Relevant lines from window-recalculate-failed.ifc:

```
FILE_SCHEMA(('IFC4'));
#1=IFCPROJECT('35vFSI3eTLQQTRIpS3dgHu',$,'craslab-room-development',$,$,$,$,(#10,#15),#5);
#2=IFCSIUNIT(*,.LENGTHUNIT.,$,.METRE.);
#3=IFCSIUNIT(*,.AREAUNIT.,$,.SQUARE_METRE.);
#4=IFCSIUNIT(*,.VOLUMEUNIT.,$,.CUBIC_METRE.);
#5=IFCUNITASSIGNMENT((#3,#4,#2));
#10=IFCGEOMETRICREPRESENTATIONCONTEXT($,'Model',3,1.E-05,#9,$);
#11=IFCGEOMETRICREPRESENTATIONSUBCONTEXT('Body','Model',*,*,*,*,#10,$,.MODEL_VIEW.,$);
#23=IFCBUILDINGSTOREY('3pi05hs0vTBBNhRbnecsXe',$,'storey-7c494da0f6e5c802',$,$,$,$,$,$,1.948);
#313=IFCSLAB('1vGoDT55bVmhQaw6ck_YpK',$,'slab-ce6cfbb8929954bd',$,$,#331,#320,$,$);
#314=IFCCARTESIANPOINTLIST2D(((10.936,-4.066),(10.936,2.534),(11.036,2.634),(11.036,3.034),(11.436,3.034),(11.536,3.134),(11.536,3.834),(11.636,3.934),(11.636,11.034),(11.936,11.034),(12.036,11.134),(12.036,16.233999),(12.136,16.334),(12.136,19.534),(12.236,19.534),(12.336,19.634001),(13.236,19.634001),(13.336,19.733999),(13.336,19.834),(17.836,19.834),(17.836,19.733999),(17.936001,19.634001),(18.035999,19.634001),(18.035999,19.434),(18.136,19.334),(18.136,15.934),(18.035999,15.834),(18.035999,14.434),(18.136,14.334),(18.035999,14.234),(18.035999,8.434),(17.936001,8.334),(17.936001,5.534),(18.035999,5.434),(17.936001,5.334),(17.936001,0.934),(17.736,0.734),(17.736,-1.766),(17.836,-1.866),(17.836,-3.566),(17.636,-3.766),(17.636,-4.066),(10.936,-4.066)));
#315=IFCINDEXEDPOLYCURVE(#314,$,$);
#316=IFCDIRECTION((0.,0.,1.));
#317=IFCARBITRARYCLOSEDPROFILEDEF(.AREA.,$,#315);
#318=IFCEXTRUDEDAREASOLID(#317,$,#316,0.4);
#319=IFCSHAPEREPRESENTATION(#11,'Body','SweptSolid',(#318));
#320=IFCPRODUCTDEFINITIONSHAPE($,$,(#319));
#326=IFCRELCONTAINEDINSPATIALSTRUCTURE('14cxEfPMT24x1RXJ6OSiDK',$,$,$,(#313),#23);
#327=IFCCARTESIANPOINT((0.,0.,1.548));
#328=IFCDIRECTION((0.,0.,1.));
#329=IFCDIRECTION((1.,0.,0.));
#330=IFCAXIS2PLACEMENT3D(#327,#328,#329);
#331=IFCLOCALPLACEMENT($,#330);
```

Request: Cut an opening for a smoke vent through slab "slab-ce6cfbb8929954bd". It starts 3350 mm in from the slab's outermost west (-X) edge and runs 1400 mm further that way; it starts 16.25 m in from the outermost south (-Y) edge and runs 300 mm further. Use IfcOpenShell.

```python
import numpy as np
import ifcopenshell
import ifcopenshell.api.feature
import ifcopenshell.api.geometry
import ifcopenshell.api.root
import ifcopenshell.geom
import ifcopenshell.util.placement
import ifcopenshell.util.representation
import ifcopenshell.util.shape
import ifcopenshell.util.unit

model = ifcopenshell.open("window-recalculate-failed.ifc")
unit_scale = ifcopenshell.util.unit.calculate_unit_scale(model)
settings = ifcopenshell.geom.settings()


def volume(element):
    """Net volume in cubic metres, openings subtracted."""
    shape = ifcopenshell.geom.create_shape(settings, element)
    return ifcopenshell.util.shape.get_volume(shape.geometry)


slab = model.by_guid("1vGoDT55bVmhQaw6ck_YpK")
before = volume(slab)

# Extent in the slab's own axes, in metres. The edges named are its -X and -Y sides.
slab_shape = ifcopenshell.geom.create_shape(settings, slab)
vertices = ifcopenshell.util.shape.get_vertices(slab_shape.geometry)
x_min, y_min, bottom = vertices.min(axis=0)
top = vertices[:, 2].max()

opening = ifcopenshell.api.root.create_entity(model, ifc_class="IfcOpeningElement", name="Smoke vent opening", predefined_type="OPENING")
context = ifcopenshell.util.representation.get_context(model, "Model", "Body", "MODEL_VIEW")
width, depth = 1.4, 0.3
outline = [(0.0, 0.0), (width, 0.0), (width, depth), (0.0, depth), (0.0, 0.0)]
# Overshoot both faces by 50 mm so the cut is clean.
shape = ifcopenshell.api.geometry.add_slab_representation(
    model, context=context, depth=top - bottom + 0.1, polyline=outline
)
ifcopenshell.api.geometry.assign_representation(model, product=opening, representation=shape)

matrix = ifcopenshell.util.placement.get_local_placement(slab.ObjectPlacement)
matrix[:, 3] = matrix @ np.append(np.array([x_min + 3.35, y_min + 16.25, bottom - 0.05]) / unit_scale, 1.0)
ifcopenshell.api.geometry.edit_object_placement(model, product=opening, matrix=matrix, is_si=False)
ifcopenshell.api.feature.add_feature(model, feature=opening, element=slab)

after = volume(slab)

print(f"slab volume {before:.3f} -> {after:.3f} m3")

model.write("window-recalculate-failed_v2.ifc")
```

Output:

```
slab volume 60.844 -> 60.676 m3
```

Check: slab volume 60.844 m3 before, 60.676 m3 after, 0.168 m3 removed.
